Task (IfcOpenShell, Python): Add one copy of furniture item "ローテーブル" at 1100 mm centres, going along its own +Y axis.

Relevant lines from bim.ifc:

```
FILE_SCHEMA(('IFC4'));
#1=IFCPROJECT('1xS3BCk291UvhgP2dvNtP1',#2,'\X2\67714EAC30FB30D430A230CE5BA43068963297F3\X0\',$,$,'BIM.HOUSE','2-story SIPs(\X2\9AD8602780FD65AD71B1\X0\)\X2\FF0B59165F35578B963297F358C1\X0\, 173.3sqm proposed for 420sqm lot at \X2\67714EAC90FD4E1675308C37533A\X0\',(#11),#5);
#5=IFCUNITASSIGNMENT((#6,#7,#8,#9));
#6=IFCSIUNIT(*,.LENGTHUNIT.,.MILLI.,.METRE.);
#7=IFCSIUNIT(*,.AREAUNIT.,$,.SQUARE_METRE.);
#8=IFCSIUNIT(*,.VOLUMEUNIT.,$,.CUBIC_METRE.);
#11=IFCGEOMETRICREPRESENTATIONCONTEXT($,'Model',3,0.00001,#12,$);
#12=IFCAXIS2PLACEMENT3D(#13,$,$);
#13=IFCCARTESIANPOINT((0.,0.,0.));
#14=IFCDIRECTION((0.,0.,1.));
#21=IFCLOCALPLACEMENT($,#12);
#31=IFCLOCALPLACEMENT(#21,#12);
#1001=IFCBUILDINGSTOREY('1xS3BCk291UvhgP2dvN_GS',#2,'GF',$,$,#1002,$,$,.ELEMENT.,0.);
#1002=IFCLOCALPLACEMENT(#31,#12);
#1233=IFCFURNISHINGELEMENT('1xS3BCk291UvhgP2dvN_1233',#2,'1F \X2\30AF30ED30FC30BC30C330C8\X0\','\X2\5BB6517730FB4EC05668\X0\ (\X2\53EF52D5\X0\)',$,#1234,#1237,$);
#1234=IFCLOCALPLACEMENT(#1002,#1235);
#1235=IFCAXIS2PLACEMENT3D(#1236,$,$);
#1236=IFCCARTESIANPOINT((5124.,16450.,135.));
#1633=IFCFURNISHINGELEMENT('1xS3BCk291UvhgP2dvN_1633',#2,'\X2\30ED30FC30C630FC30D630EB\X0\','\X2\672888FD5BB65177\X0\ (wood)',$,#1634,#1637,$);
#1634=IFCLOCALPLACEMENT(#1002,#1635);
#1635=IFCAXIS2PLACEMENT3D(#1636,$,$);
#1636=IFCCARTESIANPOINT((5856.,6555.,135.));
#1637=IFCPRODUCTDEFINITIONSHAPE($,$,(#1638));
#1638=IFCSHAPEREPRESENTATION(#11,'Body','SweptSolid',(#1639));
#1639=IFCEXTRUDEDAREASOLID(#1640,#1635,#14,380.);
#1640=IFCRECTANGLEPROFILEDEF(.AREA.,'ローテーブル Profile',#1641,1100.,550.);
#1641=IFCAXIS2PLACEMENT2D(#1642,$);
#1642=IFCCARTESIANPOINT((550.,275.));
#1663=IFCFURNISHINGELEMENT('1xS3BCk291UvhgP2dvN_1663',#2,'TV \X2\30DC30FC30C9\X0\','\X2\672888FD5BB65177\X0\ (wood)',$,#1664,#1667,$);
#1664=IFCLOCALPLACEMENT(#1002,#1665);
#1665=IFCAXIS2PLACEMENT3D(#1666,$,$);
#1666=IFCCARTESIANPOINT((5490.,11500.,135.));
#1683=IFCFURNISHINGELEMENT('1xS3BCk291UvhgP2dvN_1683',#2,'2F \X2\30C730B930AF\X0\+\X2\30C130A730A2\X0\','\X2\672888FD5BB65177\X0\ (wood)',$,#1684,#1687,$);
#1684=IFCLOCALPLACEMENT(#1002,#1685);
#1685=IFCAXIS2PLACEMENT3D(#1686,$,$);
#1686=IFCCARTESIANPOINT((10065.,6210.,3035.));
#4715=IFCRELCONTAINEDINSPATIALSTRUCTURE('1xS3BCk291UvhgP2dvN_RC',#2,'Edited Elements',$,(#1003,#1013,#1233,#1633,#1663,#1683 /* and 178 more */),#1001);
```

```python
import ifcopenshell
import ifcopenshell.api.geometry
import ifcopenshell.api.root
import ifcopenshell.util.element
import ifcopenshell.util.placement
import ifcopenshell.util.unit

model = ifcopenshell.open("bim.ifc")
unit_scale = ifcopenshell.util.unit.calculate_unit_scale(model)


def reuse_history(source, copy):
    """copy_class also copies each property set's owner history, people and application; keep the originals."""
    for rel in copy.IsDefinedBy:
        if rel.is_a("IfcRelDefinesByProperties") and (history := rel.RelatingPropertyDefinition.OwnerHistory):
            rel.RelatingPropertyDefinition.OwnerHistory = source.OwnerHistory
            ifcopenshell.util.element.remove_deep2(model, history)


source = model.by_guid("1xS3BCk291UvhgP2dvN_1633")
base = ifcopenshell.util.placement.get_local_placement(source.ObjectPlacement)
step = base[:3, 1] * 1.1 / unit_scale

for i in range(1, 2):
    copy = ifcopenshell.api.root.copy_class(model, product=source)
    copy.Representation = ifcopenshell.util.element.copy_deep(
        model, source.Representation, exclude=["IfcGeometricRepresentationContext", "IfcRepresentationMap"]
    )
    reuse_history(source, copy)
    matrix = base.copy()
    matrix[:3, 3] += i * step
    print("added at", matrix[:3, 3].round(3) + 0.0)
    ifcopenshell.api.geometry.edit_object_placement(model, product=copy, matrix=matrix, is_si=False)

model.write("bim_rev.ifc")
```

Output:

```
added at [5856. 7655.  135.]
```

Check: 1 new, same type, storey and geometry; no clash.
